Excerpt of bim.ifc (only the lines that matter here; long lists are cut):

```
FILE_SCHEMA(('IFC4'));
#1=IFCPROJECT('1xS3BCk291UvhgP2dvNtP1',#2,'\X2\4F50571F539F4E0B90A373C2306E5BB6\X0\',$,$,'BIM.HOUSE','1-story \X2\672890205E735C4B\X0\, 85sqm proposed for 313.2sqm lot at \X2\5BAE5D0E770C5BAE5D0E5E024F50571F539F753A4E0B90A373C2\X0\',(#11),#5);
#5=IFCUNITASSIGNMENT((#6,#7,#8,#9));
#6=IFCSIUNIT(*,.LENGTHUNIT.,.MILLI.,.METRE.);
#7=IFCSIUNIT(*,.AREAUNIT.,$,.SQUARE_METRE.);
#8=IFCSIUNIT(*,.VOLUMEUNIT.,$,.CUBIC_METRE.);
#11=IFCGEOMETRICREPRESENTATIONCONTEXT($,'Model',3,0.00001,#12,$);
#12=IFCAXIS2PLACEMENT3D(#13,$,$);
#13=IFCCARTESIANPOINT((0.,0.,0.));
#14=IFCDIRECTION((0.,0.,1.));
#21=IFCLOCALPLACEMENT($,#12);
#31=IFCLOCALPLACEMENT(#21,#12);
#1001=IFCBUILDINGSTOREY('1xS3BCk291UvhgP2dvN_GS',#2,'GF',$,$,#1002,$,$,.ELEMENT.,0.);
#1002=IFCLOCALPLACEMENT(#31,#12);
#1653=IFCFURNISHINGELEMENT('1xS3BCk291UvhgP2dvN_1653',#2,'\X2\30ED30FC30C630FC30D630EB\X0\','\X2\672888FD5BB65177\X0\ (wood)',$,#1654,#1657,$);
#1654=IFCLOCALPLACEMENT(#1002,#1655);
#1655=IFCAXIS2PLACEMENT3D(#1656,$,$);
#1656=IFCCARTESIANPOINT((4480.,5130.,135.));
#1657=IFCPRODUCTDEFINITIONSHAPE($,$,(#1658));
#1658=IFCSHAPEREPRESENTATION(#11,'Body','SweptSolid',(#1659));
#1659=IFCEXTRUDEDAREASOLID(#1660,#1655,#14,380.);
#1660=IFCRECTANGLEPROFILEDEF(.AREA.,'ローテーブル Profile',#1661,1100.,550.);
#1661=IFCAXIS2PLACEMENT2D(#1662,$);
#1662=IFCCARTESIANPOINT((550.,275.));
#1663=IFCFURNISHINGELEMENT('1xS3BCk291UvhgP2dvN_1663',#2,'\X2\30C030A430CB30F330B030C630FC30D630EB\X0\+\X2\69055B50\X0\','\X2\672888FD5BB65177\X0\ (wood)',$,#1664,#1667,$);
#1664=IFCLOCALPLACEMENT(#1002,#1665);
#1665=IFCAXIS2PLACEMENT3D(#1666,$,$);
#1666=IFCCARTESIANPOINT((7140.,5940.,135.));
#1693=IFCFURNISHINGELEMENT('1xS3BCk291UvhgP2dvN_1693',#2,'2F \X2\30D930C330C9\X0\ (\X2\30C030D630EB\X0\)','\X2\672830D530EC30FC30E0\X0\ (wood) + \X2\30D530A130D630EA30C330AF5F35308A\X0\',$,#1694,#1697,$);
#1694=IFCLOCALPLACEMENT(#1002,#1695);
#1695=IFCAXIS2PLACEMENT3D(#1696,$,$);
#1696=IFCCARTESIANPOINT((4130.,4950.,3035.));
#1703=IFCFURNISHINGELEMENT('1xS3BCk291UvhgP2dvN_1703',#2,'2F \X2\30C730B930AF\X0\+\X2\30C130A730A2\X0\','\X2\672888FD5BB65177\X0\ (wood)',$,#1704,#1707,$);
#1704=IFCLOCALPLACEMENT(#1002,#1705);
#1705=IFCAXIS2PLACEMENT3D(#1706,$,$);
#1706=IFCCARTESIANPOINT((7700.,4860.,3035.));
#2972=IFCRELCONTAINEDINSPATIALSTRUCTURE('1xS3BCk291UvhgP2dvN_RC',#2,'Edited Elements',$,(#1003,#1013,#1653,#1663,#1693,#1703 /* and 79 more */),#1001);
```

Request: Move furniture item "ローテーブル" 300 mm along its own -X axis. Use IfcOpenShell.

```python
import ifcopenshell
import ifcopenshell.api.geometry
import ifcopenshell.util.placement

model = ifcopenshell.open("bim.ifc")

item = model.by_id(1653)
matrix = ifcopenshell.util.placement.get_local_placement(item.ObjectPlacement)
matrix[:3, 3] -= matrix[:3, 0] * 300.0
ifcopenshell.api.geometry.edit_object_placement(model, product=item, matrix=matrix, is_si=False)

print(ifcopenshell.util.placement.get_local_placement(item.ObjectPlacement).round(3) + 0.0)

model.write("bim_v2.ifc")
```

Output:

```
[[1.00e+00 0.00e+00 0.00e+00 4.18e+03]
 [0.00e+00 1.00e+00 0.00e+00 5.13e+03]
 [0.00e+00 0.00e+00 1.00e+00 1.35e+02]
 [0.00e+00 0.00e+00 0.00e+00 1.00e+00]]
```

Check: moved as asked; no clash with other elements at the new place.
